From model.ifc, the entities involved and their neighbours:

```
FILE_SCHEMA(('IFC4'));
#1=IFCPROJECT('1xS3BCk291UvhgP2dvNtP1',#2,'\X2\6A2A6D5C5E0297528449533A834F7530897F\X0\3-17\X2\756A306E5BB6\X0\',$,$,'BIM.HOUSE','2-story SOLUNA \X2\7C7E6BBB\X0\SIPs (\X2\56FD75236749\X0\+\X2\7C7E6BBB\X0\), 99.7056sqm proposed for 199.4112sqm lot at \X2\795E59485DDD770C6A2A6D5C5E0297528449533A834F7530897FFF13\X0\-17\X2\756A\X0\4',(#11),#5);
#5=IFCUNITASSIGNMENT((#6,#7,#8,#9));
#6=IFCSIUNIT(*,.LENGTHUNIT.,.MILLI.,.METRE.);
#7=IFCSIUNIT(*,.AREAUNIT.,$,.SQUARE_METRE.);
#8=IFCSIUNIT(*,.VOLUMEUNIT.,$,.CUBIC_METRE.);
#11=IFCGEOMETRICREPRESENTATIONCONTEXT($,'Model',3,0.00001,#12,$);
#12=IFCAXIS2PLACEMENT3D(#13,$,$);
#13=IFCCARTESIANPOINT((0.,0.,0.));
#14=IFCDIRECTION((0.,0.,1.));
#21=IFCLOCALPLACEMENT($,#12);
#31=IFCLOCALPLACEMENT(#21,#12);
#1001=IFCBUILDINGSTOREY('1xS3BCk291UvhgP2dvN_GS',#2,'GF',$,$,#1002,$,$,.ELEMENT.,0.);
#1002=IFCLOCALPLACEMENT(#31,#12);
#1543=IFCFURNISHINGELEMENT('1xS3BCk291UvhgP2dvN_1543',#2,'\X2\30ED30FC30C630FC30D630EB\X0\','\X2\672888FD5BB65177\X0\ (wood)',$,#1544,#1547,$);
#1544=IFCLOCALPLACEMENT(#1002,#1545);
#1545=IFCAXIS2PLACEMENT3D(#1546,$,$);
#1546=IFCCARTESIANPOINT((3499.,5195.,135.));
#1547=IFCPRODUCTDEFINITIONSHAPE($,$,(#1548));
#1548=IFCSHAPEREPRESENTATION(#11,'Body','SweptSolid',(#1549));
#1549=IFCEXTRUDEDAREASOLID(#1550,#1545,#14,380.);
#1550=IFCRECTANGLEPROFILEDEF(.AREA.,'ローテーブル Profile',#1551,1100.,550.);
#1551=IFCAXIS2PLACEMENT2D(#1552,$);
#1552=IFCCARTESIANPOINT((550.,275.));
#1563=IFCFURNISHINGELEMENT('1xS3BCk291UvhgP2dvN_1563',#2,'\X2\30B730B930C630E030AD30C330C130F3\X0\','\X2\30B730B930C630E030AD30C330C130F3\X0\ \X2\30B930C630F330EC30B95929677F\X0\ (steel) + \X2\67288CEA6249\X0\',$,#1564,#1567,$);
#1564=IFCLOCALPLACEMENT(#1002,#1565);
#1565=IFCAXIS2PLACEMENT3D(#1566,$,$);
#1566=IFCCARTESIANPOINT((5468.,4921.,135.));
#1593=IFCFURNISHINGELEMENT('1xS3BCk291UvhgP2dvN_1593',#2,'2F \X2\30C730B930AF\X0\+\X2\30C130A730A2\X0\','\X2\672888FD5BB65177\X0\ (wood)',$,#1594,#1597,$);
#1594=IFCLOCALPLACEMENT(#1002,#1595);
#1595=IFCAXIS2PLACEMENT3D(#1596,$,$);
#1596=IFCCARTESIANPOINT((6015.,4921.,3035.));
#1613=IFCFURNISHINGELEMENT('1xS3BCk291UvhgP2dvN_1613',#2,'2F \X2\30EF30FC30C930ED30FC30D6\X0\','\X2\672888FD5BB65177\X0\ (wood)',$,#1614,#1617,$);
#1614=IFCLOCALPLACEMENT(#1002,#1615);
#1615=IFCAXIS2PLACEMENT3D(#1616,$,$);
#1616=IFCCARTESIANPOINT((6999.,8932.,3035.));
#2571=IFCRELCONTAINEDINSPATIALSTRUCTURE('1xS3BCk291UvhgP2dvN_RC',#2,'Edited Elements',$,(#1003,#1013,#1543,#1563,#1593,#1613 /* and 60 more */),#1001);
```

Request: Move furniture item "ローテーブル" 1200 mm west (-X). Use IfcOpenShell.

```python
import ifcopenshell
import ifcopenshell.api.geometry
import ifcopenshell.util.placement
import ifcopenshell.util.unit

model = ifcopenshell.open("model.ifc")
unit_scale = ifcopenshell.util.unit.calculate_unit_scale(model)

item = model.by_guid("1xS3BCk291UvhgP2dvN_1543")
matrix = ifcopenshell.util.placement.get_local_placement(item.ObjectPlacement)
matrix[0, 3] -= 1.2 / unit_scale
ifcopenshell.api.geometry.edit_object_placement(model, product=item, matrix=matrix, is_si=False)

print(ifcopenshell.util.placement.get_local_placement(item.ObjectPlacement).round(3) + 0.0)

model.write("model_edited.ifc")
```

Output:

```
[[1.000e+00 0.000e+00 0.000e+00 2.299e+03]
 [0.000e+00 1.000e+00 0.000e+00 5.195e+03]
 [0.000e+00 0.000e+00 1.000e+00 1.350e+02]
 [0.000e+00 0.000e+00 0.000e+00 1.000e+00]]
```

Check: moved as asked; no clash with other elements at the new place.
